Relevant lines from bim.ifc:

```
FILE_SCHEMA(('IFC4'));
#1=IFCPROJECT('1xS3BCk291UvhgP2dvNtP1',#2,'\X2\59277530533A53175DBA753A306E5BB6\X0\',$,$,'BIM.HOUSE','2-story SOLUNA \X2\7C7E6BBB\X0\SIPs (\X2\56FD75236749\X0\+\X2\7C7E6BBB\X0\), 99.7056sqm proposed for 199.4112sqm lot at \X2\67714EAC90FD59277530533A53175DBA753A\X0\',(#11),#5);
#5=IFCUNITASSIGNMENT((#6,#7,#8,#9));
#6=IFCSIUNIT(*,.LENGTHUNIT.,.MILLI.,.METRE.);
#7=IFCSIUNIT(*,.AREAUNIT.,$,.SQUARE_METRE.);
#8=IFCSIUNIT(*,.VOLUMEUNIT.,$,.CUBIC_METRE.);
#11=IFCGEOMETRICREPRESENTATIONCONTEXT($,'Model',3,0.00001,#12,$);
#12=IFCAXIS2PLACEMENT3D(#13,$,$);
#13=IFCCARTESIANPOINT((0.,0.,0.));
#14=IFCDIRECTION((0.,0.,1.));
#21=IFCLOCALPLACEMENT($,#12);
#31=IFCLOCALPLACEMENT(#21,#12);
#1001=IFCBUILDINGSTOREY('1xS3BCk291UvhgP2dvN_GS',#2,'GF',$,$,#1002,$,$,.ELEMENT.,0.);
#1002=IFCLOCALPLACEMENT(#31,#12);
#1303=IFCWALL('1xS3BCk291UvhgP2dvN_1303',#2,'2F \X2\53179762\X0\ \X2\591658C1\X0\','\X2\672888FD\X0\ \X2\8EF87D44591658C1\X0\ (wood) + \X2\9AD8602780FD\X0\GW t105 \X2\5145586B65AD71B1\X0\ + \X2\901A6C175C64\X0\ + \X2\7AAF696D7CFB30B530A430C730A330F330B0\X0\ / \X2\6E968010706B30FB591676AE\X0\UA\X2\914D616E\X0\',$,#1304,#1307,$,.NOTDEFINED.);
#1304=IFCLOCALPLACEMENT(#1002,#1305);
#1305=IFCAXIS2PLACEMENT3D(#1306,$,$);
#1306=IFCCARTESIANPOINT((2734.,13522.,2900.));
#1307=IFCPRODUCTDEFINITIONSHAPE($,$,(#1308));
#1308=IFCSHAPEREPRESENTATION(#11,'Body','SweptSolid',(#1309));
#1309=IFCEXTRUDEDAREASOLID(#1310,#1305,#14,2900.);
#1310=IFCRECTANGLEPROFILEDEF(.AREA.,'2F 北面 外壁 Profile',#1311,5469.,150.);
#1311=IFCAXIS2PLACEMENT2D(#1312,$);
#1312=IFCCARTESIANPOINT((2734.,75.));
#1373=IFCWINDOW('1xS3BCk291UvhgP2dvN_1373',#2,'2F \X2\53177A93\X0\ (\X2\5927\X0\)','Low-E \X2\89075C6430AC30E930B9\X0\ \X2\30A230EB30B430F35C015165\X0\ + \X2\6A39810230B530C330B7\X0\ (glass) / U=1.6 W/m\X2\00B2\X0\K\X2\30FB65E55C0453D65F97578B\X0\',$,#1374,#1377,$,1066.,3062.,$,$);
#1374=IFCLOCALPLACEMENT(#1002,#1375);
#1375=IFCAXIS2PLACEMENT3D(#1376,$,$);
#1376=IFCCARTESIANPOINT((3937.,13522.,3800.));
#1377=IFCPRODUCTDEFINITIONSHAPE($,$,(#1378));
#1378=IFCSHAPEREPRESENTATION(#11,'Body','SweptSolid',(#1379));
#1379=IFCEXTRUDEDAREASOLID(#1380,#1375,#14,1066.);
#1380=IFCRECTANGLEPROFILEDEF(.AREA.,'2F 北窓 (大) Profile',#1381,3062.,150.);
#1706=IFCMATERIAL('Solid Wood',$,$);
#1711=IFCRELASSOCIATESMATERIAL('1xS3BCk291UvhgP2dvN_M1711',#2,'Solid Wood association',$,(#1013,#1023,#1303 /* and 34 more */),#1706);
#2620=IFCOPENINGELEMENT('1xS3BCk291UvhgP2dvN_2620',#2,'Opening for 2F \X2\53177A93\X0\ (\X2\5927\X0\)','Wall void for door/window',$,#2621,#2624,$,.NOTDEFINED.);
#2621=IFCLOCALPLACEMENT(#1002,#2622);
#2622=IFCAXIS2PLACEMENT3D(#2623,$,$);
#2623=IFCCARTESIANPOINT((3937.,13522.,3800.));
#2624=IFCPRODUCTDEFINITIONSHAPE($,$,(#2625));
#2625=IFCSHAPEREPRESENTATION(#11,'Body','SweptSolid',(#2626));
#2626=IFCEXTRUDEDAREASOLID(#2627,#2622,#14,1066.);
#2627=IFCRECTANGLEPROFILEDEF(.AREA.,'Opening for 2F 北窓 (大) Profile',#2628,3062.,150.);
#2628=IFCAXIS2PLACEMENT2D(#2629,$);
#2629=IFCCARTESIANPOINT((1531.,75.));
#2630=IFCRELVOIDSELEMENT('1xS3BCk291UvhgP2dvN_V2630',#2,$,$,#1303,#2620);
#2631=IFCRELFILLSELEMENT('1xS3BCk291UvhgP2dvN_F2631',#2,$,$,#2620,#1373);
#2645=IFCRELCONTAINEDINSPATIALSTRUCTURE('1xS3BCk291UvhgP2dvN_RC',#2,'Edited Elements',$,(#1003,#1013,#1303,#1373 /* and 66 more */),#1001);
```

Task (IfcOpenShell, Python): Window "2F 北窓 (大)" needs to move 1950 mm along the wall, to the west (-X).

```python
import ifcopenshell
import ifcopenshell.api.geometry
import ifcopenshell.util.placement

model = ifcopenshell.open("bim.ifc")

window = model.by_guid("1xS3BCk291UvhgP2dvN_1373")
opening = window.FillsVoids[0].RelatingOpeningElement
wall = opening.VoidsElements[0].RelatingBuildingElement

wall_matrix = ifcopenshell.util.placement.get_local_placement(wall.ObjectPlacement)
shift = wall_matrix[:3, 0] * -1950.0
before = ifcopenshell.util.placement.get_local_placement(window.ObjectPlacement)[:3, 3].copy()

# The window is not placed relative to its opening, so move both.
for product in (opening, window):
    matrix = ifcopenshell.util.placement.get_local_placement(product.ObjectPlacement)
    matrix[:3, 3] += shift
    ifcopenshell.api.geometry.edit_object_placement(model, product=product, matrix=matrix, is_si=False)

after = ifcopenshell.util.placement.get_local_placement(window.ObjectPlacement)[:3, 3]
print("window moved by", (after - before).round(3) + 0.0)

model.write("bim_updated.ifc")
```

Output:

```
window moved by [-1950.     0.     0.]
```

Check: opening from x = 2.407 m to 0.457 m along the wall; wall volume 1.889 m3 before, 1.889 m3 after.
